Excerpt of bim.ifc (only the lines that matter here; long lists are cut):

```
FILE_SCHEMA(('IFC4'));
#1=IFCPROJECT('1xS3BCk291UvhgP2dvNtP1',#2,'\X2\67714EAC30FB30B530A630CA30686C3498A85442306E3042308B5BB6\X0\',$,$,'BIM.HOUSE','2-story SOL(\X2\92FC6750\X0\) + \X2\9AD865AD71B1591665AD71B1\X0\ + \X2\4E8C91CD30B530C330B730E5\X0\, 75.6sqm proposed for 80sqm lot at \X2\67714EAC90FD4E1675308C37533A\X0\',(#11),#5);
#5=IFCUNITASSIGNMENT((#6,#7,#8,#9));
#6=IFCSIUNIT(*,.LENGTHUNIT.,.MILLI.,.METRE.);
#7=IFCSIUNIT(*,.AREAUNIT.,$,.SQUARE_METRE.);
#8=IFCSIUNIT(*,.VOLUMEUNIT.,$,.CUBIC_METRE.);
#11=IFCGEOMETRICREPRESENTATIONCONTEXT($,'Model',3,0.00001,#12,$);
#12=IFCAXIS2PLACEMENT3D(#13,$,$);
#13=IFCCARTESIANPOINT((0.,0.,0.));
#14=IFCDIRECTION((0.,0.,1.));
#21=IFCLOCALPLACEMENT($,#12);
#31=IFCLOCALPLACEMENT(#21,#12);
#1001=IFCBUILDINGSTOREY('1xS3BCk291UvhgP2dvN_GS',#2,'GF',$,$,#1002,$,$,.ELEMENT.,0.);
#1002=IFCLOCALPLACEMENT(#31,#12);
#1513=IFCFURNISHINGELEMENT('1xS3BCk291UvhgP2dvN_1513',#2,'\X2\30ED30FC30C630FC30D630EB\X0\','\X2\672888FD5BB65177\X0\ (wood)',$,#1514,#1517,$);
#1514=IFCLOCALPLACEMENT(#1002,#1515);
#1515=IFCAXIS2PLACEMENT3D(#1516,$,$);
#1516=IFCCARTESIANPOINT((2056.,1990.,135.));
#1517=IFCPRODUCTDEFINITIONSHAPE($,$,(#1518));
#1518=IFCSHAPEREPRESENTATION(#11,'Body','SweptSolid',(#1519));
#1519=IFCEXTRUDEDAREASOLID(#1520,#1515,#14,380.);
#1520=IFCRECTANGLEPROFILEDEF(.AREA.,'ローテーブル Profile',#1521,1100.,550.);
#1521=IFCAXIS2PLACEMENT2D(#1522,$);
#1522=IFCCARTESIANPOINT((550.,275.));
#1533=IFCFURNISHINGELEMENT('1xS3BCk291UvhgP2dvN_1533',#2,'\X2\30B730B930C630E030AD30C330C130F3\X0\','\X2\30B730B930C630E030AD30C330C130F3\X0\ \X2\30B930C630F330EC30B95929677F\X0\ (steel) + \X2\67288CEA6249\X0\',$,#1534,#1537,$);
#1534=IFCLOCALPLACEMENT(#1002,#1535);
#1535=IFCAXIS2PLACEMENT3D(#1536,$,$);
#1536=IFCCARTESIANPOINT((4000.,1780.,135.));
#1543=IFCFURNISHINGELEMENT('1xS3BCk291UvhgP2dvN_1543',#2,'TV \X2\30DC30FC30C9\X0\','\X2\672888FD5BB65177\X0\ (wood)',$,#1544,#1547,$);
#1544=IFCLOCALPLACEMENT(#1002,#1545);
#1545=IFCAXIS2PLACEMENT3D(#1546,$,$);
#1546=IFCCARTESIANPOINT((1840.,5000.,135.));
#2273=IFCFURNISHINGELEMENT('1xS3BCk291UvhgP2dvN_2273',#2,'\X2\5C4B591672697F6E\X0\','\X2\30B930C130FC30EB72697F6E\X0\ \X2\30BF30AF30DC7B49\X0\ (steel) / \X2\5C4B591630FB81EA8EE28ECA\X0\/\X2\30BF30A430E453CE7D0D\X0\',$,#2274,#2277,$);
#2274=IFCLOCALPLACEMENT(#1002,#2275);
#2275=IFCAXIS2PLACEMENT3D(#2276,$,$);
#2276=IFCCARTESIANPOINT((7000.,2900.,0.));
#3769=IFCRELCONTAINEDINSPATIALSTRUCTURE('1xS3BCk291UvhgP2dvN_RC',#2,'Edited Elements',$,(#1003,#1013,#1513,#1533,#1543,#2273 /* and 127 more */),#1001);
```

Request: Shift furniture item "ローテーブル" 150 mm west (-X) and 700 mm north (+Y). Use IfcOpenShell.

```python
import ifcopenshell
import ifcopenshell.api.geometry
import ifcopenshell.util.placement
import ifcopenshell.util.unit

model = ifcopenshell.open("bim.ifc")
unit_scale = ifcopenshell.util.unit.calculate_unit_scale(model)

item = model.by_guid("1xS3BCk291UvhgP2dvN_1513")
matrix = ifcopenshell.util.placement.get_local_placement(item.ObjectPlacement)
matrix[0, 3] -= 0.15 / unit_scale
matrix[1, 3] += 0.7 / unit_scale
ifcopenshell.api.geometry.edit_object_placement(model, product=item, matrix=matrix, is_si=False)

print(ifcopenshell.util.placement.get_local_placement(item.ObjectPlacement).round(3) + 0.0)

model.write("bim_rev.ifc")
```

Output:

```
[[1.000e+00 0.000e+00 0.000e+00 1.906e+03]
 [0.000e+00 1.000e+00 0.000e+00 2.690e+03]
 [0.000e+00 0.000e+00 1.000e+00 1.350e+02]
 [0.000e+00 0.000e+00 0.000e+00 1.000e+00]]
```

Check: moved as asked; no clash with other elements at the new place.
